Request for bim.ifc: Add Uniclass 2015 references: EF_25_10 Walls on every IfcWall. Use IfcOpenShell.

First a look at what the model holds.

```python
import ifcopenshell

model = ifcopenshell.open("bim.ifc")
print(model.schema)
print("classifications:", [c.Name for c in model.by_type("IfcClassification")])
for ifc_class in ("IfcDoor", "IfcRoof", "IfcStair", "IfcWall", "IfcWindow"):
    print(ifc_class, len(model.by_type(ifc_class)))
```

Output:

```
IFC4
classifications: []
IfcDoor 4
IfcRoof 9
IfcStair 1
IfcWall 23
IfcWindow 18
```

```python
import ifcopenshell
import ifcopenshell.api.classification

model = ifcopenshell.open("bim.ifc")

system = ifcopenshell.api.classification.add_classification(model, classification="Uniclass 2015")

codes = {
    "IfcWall": ("EF_25_10", "Walls"),
}
for ifc_class, (code, name) in codes.items():
    products = model.by_type(ifc_class)
    ifcopenshell.api.classification.add_reference(
        model, products=products, classification=system, identification=code, name=name
    )
    print(code, len(products))

model.write("bim_v2.ifc")
```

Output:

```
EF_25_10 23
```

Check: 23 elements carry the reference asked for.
